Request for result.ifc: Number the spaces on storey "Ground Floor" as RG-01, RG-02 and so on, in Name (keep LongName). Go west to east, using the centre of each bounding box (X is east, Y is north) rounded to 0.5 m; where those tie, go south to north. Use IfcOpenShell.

First a look at what the model holds.

```python
import ifcopenshell
import ifcopenshell.util.element
import ifcopenshell.util.placement

model = ifcopenshell.open("result.ifc")
print(model.schema)
storey = next(s for s in model.by_type("IfcBuildingStorey") if s.Name == "Ground Floor")
spaces = [e for e in ifcopenshell.util.element.get_decomposition(storey) if e.is_a("IfcSpace")]
for e in sorted(spaces, key=lambda e: e.id()):
    origin = ifcopenshell.util.placement.get_local_placement(e.ObjectPlacement)[:3, 3]
    print(e.id(), e.Name, e.LongName, origin.round(2) + 0.0, sep=" | ")
```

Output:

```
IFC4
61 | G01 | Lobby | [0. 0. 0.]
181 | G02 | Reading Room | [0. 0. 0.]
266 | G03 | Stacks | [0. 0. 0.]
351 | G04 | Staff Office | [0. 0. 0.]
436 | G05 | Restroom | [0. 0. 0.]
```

```python
import ifcopenshell
import ifcopenshell.geom
import ifcopenshell.util.element
import ifcopenshell.util.shape

model = ifcopenshell.open("result.ifc")
settings = ifcopenshell.geom.settings()
settings.set("use-world-coords", True)


def centre(element):
    shape = ifcopenshell.geom.create_shape(settings, element)
    return ifcopenshell.util.shape.get_bbox_centroid(shape.geometry)


storey = next(s for s in model.by_type("IfcBuildingStorey") if s.Name == "Ground Floor")
spaces = [e for e in ifcopenshell.util.element.get_decomposition(storey) if e.is_a("IfcSpace")]

# Insertion points can sit at a corner or the storey origin, so sort by the geometry (in metres).
centres = {e: centre(e) for e in spaces}
spaces.sort(key=lambda e: (round(centres[e][0] / 0.5), centres[e][1]))

for i, e in enumerate(spaces, start=1):
    number = f"RG-{i:02d}"
    e.Name = number
    print(e.id(), number)

model.write("result-out.ifc")
```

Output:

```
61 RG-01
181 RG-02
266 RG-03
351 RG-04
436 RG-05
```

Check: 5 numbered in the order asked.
